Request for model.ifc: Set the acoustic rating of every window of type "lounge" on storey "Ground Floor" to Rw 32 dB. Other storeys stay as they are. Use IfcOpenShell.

First a look at what the model holds.

```python
import ifcopenshell
import ifcopenshell.util.element

model = ifcopenshell.open("model.ifc")
print(model.schema)
storey = next(s for s in model.by_type("IfcBuildingStorey") if s.Name == "Ground Floor")
windows = [e for e in ifcopenshell.util.element.get_decomposition(storey) if e.is_a("IfcWindow")]
seen = {}
for e in windows:
    element_type = ifcopenshell.util.element.get_type(e)
    key = (element_type.Name if element_type != e and element_type else None, ifcopenshell.util.element.get_pset(e, "Pset_WindowCommon", "AcousticRating"))
    seen[key] = seen.get(key, 0) + 1
for (name, value), count in sorted(seen.items(), key=str):
    print(count, "x", name, "|", value)
```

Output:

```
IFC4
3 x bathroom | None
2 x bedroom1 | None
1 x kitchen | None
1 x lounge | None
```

```python
import ifcopenshell
import ifcopenshell.api.pset
import ifcopenshell.util.element

model = ifcopenshell.open("model.ifc")

storey = next(s for s in model.by_type("IfcBuildingStorey") if s.Name == "Ground Floor")
windows = [e for e in ifcopenshell.util.element.get_decomposition(storey) if e.is_a("IfcWindow")]

count = 0
for e in windows:
    element_type = ifcopenshell.util.element.get_type(e)
    if element_type in (None, e) or element_type.Name != "lounge":
        continue
    # add_pset returns the element's existing set when there is one.
    pset = ifcopenshell.api.pset.add_pset(model, product=e, name="Pset_WindowCommon")
    ifcopenshell.api.pset.edit_pset(model, pset=pset, properties={"AcousticRating": "Rw 32 dB"})
    count += 1

print(count, "windows updated")

model.write("model_v2.ifc")
```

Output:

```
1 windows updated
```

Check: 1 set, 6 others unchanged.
